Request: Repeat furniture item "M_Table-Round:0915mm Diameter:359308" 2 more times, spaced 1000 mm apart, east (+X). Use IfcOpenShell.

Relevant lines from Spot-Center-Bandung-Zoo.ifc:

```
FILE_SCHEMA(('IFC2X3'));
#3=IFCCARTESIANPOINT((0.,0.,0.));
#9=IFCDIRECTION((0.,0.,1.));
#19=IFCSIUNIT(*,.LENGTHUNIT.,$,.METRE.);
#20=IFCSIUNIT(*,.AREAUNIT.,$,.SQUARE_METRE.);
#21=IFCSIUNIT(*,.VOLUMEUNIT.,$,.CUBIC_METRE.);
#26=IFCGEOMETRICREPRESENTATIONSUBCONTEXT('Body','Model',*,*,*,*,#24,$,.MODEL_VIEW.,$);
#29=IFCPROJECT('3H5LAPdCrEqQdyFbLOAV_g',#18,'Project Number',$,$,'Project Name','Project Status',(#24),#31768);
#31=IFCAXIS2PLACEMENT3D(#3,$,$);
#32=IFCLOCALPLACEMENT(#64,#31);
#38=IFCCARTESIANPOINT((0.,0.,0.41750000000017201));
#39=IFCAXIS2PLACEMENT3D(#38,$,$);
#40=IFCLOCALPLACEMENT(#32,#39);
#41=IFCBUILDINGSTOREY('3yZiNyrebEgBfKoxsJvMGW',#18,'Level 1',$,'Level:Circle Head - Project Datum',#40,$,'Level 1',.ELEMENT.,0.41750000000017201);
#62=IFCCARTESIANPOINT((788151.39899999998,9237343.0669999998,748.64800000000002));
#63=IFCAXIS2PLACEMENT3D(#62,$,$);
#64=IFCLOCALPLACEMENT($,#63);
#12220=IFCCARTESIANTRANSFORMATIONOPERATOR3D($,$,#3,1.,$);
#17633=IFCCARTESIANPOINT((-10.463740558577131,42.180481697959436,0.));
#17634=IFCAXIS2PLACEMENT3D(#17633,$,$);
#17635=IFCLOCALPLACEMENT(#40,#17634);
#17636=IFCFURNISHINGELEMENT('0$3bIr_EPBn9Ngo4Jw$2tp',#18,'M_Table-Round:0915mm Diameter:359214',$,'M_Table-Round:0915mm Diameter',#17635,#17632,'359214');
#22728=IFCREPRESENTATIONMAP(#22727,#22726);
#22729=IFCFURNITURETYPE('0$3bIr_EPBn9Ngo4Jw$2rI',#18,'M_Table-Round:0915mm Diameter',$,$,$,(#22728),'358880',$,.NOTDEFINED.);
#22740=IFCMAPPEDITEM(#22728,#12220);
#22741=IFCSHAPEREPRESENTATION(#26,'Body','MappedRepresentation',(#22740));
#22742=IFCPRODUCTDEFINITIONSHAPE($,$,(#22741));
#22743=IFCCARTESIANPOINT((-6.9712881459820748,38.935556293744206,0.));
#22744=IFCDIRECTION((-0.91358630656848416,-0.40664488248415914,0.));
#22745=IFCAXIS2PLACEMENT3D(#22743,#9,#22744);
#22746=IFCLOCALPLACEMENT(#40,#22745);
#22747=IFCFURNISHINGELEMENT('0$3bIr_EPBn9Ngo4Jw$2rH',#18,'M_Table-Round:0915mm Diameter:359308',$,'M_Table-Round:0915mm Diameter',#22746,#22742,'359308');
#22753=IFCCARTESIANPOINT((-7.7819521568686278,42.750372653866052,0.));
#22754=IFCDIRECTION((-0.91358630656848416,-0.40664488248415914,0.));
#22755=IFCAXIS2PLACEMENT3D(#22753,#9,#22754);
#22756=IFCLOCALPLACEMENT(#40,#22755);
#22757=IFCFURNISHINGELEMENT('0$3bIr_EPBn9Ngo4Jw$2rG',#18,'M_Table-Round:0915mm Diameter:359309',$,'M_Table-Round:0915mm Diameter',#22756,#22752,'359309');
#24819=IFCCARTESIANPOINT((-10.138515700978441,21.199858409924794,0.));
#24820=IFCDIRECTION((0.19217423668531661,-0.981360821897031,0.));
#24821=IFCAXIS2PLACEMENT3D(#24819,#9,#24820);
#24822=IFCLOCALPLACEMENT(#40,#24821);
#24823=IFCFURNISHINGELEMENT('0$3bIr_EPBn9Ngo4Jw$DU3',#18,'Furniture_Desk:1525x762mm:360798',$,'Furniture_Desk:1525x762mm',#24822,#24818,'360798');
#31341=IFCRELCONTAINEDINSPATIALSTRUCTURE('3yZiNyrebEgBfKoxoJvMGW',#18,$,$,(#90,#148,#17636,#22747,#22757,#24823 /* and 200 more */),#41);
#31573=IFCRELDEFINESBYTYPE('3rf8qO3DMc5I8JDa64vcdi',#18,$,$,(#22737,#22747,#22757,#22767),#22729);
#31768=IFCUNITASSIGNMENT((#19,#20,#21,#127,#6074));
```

```python
import numpy as np
import ifcopenshell
import ifcopenshell.api.geometry
import ifcopenshell.api.root
import ifcopenshell.util.element
import ifcopenshell.util.placement
import ifcopenshell.util.unit

model = ifcopenshell.open("Spot-Center-Bandung-Zoo.ifc")
unit_scale = ifcopenshell.util.unit.calculate_unit_scale(model)


def reuse_history(source, copy):
    """copy_class also copies each property set's owner history, people and application; keep the originals."""
    for rel in copy.IsDefinedBy:
        if rel.is_a("IfcRelDefinesByProperties") and (history := rel.RelatingPropertyDefinition.OwnerHistory):
            rel.RelatingPropertyDefinition.OwnerHistory = source.OwnerHistory
            ifcopenshell.util.element.remove_deep2(model, history)


source = model.by_id(22747)
base = ifcopenshell.util.placement.get_local_placement(source.ObjectPlacement)
step = np.array([1.0, 0.0, 0.0]) * 1 / unit_scale

for i in range(1, 3):
    copy = ifcopenshell.api.root.copy_class(model, product=source)
    copy.Representation = ifcopenshell.util.element.copy_deep(
        model, source.Representation, exclude=["IfcGeometricRepresentationContext", "IfcRepresentationMap"]
    )
    copy.Name = "M_Table-Round:0915mm Diameter"
    copy.Tag = None
    reuse_history(source, copy)
    matrix = base.copy()
    matrix[:3, 3] += i * step
    print("added at", matrix[:3, 3].round(3) + 0.0)
    ifcopenshell.api.geometry.edit_object_placement(model, product=copy, matrix=matrix, is_si=False)

model.write("Spot-Center-Bandung-Zoo_v2.ifc")
```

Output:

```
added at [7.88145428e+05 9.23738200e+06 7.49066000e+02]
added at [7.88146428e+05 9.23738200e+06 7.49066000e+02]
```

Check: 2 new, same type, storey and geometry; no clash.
